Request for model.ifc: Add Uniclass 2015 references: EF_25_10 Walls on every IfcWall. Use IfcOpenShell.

First a look at what the model holds.

```python
import ifcopenshell

model = ifcopenshell.open("model.ifc")
print(model.schema)
print("classifications:", [c.Name for c in model.by_type("IfcClassification")])
for ifc_class in ("IfcDoor", "IfcRoof", "IfcStair", "IfcWall", "IfcWindow"):
    print(ifc_class, len(model.by_type(ifc_class)))
```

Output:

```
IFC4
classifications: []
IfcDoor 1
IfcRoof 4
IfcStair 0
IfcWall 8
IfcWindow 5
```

```python
import ifcopenshell
import ifcopenshell.api.classification

model = ifcopenshell.open("model.ifc")

system = ifcopenshell.api.classification.add_classification(model, classification="Uniclass 2015")

codes = {
    "IfcWall": ("EF_25_10", "Walls"),
}
for ifc_class, (code, name) in codes.items():
    products = model.by_type(ifc_class)
    ifcopenshell.api.classification.add_reference(
        model, products=products, classification=system, identification=code, name=name
    )
    print(code, len(products))

model.write("model_edited.ifc")
```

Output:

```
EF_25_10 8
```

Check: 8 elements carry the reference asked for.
